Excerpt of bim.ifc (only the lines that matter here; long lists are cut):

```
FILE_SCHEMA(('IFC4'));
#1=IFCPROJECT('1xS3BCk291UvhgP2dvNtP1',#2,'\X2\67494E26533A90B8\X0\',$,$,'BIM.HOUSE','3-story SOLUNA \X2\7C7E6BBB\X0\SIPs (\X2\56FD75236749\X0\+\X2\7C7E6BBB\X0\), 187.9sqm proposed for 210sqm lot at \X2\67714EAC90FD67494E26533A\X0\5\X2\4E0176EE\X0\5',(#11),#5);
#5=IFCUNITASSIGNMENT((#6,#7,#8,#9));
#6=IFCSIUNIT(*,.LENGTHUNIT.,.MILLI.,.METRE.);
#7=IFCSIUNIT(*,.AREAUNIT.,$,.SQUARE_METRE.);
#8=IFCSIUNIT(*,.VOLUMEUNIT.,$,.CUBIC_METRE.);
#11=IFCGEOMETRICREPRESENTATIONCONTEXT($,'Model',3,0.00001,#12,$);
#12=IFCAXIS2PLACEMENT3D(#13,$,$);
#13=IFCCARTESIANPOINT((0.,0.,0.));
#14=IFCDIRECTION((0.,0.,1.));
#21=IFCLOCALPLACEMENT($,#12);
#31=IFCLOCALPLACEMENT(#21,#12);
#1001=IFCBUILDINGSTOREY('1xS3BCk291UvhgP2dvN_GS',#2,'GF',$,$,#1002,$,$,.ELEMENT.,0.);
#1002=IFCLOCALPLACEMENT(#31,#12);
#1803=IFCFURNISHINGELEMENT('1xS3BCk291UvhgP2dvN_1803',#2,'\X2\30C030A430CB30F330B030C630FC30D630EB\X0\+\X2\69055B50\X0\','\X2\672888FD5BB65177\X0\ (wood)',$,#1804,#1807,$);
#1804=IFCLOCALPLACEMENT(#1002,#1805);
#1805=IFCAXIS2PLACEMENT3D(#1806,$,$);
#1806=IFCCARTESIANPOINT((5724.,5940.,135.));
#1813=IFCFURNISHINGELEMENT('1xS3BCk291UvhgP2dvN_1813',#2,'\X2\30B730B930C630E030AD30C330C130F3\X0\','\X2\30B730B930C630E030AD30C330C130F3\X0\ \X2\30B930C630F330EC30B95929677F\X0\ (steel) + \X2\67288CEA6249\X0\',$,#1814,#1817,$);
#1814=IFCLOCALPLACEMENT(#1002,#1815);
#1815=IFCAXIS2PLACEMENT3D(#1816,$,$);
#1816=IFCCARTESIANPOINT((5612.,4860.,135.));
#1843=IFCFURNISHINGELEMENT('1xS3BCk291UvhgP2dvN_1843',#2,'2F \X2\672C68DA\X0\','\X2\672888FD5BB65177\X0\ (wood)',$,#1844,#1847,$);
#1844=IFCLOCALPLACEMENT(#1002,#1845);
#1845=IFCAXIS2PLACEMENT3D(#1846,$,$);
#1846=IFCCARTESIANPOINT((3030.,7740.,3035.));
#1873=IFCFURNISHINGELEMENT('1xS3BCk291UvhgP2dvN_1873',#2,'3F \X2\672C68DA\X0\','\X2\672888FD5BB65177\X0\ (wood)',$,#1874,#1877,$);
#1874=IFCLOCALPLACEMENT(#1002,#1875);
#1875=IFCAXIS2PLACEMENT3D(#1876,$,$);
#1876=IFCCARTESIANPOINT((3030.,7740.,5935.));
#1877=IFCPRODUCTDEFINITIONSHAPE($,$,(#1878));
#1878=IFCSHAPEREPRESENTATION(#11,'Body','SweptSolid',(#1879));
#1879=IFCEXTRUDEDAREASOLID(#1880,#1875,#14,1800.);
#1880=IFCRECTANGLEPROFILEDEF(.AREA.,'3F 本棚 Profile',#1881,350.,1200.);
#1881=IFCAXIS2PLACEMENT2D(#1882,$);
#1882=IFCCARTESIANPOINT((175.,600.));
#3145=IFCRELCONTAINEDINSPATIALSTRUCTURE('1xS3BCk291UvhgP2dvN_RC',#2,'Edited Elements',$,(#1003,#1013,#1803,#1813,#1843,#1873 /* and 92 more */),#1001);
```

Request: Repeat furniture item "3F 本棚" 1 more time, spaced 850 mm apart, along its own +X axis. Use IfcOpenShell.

```python
import ifcopenshell
import ifcopenshell.api.geometry
import ifcopenshell.api.root
import ifcopenshell.util.element
import ifcopenshell.util.placement
import ifcopenshell.util.unit

model = ifcopenshell.open("bim.ifc")
unit_scale = ifcopenshell.util.unit.calculate_unit_scale(model)


def reuse_history(source, copy):
    """copy_class also copies each property set's owner history, people and application; keep the originals."""
    for rel in copy.IsDefinedBy:
        if rel.is_a("IfcRelDefinesByProperties") and (history := rel.RelatingPropertyDefinition.OwnerHistory):
            rel.RelatingPropertyDefinition.OwnerHistory = source.OwnerHistory
            ifcopenshell.util.element.remove_deep2(model, history)


source = model.by_guid("1xS3BCk291UvhgP2dvN_1873")
base = ifcopenshell.util.placement.get_local_placement(source.ObjectPlacement)
step = base[:3, 0] * 0.85 / unit_scale

for i in range(1, 2):
    copy = ifcopenshell.api.root.copy_class(model, product=source)
    copy.Representation = ifcopenshell.util.element.copy_deep(
        model, source.Representation, exclude=["IfcGeometricRepresentationContext", "IfcRepresentationMap"]
    )
    reuse_history(source, copy)
    matrix = base.copy()
    matrix[:3, 3] += i * step
    print("added at", matrix[:3, 3].round(3) + 0.0)
    ifcopenshell.api.geometry.edit_object_placement(model, product=copy, matrix=matrix, is_si=False)

model.write("bim_v2.ifc")
```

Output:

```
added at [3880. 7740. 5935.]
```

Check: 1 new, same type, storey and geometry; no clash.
